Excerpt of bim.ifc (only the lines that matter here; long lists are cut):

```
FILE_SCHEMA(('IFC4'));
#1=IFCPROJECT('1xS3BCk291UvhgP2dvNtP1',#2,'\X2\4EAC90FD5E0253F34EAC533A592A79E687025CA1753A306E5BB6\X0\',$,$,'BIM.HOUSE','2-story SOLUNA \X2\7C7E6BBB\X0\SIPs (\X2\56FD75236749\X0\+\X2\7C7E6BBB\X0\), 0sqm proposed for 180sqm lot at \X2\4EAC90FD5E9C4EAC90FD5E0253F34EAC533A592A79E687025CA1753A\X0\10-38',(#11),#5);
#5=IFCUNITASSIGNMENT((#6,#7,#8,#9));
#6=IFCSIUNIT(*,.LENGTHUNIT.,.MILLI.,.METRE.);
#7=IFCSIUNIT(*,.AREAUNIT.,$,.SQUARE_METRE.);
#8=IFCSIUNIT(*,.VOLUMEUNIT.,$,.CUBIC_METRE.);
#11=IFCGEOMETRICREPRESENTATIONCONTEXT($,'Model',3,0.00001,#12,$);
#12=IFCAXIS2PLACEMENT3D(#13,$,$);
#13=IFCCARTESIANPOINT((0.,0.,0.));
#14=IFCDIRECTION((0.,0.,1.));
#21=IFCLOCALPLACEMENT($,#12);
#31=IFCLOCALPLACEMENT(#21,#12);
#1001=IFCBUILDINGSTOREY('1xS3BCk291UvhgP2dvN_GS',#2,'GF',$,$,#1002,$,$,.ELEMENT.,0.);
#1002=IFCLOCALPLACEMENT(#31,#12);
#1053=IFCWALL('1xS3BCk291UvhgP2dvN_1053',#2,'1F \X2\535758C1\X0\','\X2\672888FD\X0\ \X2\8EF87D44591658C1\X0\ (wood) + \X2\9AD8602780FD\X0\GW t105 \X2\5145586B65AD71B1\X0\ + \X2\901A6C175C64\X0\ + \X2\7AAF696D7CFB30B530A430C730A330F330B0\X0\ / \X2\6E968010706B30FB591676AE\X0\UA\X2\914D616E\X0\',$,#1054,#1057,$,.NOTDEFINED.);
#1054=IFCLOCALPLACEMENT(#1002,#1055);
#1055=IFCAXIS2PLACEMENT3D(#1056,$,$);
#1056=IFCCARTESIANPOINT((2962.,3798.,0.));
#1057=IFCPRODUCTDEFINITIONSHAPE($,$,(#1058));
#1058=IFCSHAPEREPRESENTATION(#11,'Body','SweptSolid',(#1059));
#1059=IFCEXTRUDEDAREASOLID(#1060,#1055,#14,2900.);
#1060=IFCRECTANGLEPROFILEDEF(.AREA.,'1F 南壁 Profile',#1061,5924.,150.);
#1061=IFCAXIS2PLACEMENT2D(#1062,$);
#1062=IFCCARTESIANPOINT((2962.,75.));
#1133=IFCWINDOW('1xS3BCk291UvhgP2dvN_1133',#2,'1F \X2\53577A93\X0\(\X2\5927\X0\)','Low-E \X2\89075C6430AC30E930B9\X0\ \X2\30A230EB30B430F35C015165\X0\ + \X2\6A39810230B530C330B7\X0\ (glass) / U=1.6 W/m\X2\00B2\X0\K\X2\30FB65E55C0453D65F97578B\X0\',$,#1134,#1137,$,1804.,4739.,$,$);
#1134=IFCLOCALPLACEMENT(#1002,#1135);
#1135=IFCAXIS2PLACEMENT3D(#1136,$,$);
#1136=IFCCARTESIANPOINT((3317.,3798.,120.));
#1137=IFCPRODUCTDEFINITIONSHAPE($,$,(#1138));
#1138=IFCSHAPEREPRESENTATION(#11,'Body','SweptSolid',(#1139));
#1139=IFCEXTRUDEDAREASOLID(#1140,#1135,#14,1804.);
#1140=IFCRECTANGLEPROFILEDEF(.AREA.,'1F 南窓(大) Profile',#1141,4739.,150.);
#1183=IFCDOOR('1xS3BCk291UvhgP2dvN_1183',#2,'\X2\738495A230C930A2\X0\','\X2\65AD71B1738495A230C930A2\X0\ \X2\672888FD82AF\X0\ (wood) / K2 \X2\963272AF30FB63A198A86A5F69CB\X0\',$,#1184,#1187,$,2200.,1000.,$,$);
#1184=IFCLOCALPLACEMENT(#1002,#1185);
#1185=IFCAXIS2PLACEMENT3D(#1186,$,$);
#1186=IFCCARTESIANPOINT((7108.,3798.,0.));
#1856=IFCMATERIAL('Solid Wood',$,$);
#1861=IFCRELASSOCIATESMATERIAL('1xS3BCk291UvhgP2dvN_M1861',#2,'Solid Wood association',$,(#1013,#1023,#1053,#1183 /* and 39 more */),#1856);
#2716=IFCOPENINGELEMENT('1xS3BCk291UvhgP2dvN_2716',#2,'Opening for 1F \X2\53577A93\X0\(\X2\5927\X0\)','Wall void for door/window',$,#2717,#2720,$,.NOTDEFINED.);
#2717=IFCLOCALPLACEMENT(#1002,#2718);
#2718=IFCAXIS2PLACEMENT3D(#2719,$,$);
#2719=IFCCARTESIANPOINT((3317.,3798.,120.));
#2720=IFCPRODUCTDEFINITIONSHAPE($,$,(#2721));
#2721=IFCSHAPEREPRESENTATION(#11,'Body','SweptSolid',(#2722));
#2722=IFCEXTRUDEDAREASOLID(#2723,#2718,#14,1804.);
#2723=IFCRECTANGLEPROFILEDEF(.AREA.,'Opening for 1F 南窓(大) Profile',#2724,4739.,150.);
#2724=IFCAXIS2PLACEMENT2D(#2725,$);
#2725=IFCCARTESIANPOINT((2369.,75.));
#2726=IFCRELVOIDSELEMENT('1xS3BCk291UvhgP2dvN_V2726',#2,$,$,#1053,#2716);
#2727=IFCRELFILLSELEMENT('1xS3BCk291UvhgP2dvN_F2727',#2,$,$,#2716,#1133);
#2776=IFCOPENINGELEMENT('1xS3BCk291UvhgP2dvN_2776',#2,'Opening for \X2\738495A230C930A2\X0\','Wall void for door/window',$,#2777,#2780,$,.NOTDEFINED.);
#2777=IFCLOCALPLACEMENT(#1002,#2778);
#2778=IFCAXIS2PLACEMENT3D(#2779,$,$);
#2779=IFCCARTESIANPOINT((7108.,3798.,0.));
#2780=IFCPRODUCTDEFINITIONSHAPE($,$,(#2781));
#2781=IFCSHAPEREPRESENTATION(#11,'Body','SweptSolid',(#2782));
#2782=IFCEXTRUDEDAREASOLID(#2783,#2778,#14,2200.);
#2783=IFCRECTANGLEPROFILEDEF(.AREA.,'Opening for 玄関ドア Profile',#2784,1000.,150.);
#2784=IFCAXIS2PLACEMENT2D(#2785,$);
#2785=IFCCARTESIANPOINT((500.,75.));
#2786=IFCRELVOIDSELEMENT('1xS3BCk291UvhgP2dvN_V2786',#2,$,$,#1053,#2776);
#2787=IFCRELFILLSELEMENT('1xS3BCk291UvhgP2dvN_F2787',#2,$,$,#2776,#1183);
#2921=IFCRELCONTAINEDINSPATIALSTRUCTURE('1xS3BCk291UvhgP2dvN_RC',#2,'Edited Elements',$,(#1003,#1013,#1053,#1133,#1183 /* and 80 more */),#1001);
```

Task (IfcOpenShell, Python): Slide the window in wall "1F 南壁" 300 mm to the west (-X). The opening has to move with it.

```python
import ifcopenshell
import ifcopenshell.api.geometry
import ifcopenshell.util.placement
import ifcopenshell.util.unit

model = ifcopenshell.open("bim.ifc")
unit_scale = ifcopenshell.util.unit.calculate_unit_scale(model)

window = model.by_guid("1xS3BCk291UvhgP2dvN_1133")
opening = window.FillsVoids[0].RelatingOpeningElement
wall = opening.VoidsElements[0].RelatingBuildingElement

wall_matrix = ifcopenshell.util.placement.get_local_placement(wall.ObjectPlacement)
shift = wall_matrix[:3, 0] * -0.3 / unit_scale
before = ifcopenshell.util.placement.get_local_placement(window.ObjectPlacement)[:3, 3].copy()

# The window is not placed relative to its opening, so move both.
for product in (opening, window):
    matrix = ifcopenshell.util.placement.get_local_placement(product.ObjectPlacement)
    matrix[:3, 3] += shift
    ifcopenshell.api.geometry.edit_object_placement(model, product=product, matrix=matrix, is_si=False)

after = ifcopenshell.util.placement.get_local_placement(window.ObjectPlacement)[:3, 3]
print("window moved by", (after - before).round(3) + 0.0)

model.write("bim-out.ifc")
```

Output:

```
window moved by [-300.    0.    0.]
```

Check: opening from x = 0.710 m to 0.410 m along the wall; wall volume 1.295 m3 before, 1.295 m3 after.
